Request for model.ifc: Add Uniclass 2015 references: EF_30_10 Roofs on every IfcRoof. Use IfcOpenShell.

First a look at what the model holds.

```python
import ifcopenshell

model = ifcopenshell.open("model.ifc")
print(model.schema)
print("classifications:", [c.Name for c in model.by_type("IfcClassification")])
for ifc_class in ("IfcDoor", "IfcRoof", "IfcStair", "IfcWall", "IfcWindow"):
    print(ifc_class, len(model.by_type(ifc_class)))
```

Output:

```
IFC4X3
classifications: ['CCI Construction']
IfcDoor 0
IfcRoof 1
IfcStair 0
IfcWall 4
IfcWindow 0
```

```python
import ifcopenshell
import ifcopenshell.api.classification

model = ifcopenshell.open("model.ifc")

system = ifcopenshell.api.classification.add_classification(model, classification="Uniclass 2015")

codes = {
    "IfcRoof": ("EF_30_10", "Roofs"),
}
for ifc_class, (code, name) in codes.items():
    products = model.by_type(ifc_class)
    ifcopenshell.api.classification.add_reference(
        model, products=products, classification=system, identification=code, name=name
    )
    print(code, len(products))

model.write("model_edited.ifc")
```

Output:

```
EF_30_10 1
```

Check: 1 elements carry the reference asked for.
